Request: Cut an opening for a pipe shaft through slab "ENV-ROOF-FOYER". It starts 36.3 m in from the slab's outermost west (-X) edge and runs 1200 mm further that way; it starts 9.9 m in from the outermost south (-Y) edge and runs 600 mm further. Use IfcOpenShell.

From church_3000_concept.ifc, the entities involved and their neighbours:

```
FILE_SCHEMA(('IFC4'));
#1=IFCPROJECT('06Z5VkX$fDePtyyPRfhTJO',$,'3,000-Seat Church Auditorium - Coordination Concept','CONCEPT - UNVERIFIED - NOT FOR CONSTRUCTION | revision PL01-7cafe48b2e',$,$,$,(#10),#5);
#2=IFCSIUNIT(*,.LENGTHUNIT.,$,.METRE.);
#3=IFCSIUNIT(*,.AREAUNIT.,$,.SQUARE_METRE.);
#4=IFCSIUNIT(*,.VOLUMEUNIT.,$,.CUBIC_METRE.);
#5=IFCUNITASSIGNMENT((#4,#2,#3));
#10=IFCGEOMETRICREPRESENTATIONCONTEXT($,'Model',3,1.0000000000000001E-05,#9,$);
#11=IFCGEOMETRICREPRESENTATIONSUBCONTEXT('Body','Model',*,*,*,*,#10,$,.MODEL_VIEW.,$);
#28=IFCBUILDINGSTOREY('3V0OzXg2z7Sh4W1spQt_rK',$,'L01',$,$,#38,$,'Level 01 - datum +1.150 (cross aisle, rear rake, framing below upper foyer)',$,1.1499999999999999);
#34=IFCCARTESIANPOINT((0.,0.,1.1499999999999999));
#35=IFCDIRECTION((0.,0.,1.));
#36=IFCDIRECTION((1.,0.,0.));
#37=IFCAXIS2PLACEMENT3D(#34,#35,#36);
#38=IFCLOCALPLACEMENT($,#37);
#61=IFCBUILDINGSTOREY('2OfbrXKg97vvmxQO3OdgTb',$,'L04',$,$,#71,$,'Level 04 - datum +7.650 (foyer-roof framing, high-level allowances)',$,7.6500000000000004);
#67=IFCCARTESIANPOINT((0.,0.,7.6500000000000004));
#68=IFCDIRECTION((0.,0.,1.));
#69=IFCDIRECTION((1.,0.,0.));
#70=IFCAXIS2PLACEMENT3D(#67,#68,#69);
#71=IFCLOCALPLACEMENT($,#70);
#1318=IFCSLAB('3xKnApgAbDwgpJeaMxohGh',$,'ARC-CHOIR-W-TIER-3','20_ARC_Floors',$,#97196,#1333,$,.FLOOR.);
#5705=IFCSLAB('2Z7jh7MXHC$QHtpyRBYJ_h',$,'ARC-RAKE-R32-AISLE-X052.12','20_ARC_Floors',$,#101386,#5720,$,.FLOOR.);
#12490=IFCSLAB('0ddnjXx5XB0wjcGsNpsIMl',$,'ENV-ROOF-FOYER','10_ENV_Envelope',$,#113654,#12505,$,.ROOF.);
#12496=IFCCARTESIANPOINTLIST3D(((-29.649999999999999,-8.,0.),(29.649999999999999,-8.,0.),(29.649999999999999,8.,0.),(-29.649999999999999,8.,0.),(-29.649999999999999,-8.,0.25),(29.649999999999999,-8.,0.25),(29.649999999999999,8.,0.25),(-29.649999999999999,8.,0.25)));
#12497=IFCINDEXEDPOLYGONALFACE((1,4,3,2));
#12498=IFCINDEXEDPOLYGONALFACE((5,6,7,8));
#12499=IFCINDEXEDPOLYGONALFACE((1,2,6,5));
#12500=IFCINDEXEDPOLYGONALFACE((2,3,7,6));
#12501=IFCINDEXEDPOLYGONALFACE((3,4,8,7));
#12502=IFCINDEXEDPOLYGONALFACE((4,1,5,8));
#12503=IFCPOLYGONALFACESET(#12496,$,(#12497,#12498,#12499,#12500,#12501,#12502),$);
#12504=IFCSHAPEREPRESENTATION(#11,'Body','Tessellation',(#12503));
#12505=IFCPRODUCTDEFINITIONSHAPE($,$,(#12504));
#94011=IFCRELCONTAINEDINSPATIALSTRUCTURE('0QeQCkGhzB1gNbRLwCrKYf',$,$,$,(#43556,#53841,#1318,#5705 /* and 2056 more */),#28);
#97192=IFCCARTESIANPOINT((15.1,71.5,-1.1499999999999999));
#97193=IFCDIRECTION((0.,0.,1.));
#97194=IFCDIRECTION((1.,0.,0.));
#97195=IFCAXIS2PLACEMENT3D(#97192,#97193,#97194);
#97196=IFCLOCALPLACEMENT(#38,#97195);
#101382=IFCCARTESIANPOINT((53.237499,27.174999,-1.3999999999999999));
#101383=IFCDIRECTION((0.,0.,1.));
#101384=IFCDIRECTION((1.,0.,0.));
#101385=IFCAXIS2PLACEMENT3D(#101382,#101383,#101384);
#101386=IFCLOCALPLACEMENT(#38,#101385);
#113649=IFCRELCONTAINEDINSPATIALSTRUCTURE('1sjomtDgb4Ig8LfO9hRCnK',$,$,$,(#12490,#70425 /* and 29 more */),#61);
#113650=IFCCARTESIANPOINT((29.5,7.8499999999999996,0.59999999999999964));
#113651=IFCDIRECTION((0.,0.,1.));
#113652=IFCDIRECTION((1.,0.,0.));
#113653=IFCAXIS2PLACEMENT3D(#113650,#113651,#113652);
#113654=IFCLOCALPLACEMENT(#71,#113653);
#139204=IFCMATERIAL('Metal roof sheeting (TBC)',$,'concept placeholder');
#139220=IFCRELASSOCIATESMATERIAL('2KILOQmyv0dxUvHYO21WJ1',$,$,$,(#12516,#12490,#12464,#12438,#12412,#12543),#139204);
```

```python
import numpy as np
import ifcopenshell
import ifcopenshell.api.feature
import ifcopenshell.api.geometry
import ifcopenshell.api.root
import ifcopenshell.geom
import ifcopenshell.util.placement
import ifcopenshell.util.representation
import ifcopenshell.util.shape
import ifcopenshell.util.unit

model = ifcopenshell.open("church_3000_concept.ifc")
unit_scale = ifcopenshell.util.unit.calculate_unit_scale(model)
settings = ifcopenshell.geom.settings()


def volume(element):
    """Net volume in cubic metres, openings subtracted."""
    shape = ifcopenshell.geom.create_shape(settings, element)
    return ifcopenshell.util.shape.get_volume(shape.geometry)


slab = model.by_guid("0ddnjXx5XB0wjcGsNpsIMl")
before = volume(slab)

# Extent in the slab's own axes, in metres. The edges named are its -X and -Y sides.
slab_shape = ifcopenshell.geom.create_shape(settings, slab)
vertices = ifcopenshell.util.shape.get_vertices(slab_shape.geometry)
x_min, y_min, bottom = vertices.min(axis=0)
top = vertices[:, 2].max()

opening = ifcopenshell.api.root.create_entity(model, ifc_class="IfcOpeningElement", name="Pipe shaft opening", predefined_type="OPENING")
context = ifcopenshell.util.representation.get_context(model, "Model", "Body", "MODEL_VIEW")
width, depth = 1.2, 0.6
outline = [(0.0, 0.0), (width, 0.0), (width, depth), (0.0, depth), (0.0, 0.0)]
# Overshoot both faces by 50 mm so the cut is clean.
shape = ifcopenshell.api.geometry.add_slab_representation(
    model, context=context, depth=top - bottom + 0.1, polyline=outline
)
ifcopenshell.api.geometry.assign_representation(model, product=opening, representation=shape)

matrix = ifcopenshell.util.placement.get_local_placement(slab.ObjectPlacement)
matrix[:, 3] = matrix @ np.append(np.array([x_min + 36.3, y_min + 9.9, bottom - 0.05]) / unit_scale, 1.0)
ifcopenshell.api.geometry.edit_object_placement(model, product=opening, matrix=matrix, is_si=False)
ifcopenshell.api.feature.add_feature(model, feature=opening, element=slab)

after = volume(slab)

print(f"slab volume {before:.3f} -> {after:.3f} m3")

model.write("church_3000_concept_updated.ifc")
```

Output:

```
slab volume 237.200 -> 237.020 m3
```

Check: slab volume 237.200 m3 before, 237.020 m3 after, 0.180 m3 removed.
